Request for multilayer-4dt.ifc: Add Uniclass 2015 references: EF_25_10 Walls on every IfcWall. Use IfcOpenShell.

First a look at what the model holds.

```python
import ifcopenshell

model = ifcopenshell.open("multilayer-4dt.ifc")
print(model.schema)
print("classifications:", [c.Name for c in model.by_type("IfcClassification")])
for ifc_class in ("IfcDoor", "IfcRoof", "IfcStair", "IfcWall", "IfcWindow"):
    print(ifc_class, len(model.by_type(ifc_class)))
```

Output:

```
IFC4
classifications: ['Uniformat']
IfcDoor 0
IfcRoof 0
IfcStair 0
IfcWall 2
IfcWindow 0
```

```python
import ifcopenshell
import ifcopenshell.api.classification

model = ifcopenshell.open("multilayer-4dt.ifc")

system = ifcopenshell.api.classification.add_classification(model, classification="Uniclass 2015")

codes = {
    "IfcWall": ("EF_25_10", "Walls"),
}
for ifc_class, (code, name) in codes.items():
    products = model.by_type(ifc_class)
    ifcopenshell.api.classification.add_reference(
        model, products=products, classification=system, identification=code, name=name
    )
    print(code, len(products))

model.write("multilayer-4dt-out.ifc")
```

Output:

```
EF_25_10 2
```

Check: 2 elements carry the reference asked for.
